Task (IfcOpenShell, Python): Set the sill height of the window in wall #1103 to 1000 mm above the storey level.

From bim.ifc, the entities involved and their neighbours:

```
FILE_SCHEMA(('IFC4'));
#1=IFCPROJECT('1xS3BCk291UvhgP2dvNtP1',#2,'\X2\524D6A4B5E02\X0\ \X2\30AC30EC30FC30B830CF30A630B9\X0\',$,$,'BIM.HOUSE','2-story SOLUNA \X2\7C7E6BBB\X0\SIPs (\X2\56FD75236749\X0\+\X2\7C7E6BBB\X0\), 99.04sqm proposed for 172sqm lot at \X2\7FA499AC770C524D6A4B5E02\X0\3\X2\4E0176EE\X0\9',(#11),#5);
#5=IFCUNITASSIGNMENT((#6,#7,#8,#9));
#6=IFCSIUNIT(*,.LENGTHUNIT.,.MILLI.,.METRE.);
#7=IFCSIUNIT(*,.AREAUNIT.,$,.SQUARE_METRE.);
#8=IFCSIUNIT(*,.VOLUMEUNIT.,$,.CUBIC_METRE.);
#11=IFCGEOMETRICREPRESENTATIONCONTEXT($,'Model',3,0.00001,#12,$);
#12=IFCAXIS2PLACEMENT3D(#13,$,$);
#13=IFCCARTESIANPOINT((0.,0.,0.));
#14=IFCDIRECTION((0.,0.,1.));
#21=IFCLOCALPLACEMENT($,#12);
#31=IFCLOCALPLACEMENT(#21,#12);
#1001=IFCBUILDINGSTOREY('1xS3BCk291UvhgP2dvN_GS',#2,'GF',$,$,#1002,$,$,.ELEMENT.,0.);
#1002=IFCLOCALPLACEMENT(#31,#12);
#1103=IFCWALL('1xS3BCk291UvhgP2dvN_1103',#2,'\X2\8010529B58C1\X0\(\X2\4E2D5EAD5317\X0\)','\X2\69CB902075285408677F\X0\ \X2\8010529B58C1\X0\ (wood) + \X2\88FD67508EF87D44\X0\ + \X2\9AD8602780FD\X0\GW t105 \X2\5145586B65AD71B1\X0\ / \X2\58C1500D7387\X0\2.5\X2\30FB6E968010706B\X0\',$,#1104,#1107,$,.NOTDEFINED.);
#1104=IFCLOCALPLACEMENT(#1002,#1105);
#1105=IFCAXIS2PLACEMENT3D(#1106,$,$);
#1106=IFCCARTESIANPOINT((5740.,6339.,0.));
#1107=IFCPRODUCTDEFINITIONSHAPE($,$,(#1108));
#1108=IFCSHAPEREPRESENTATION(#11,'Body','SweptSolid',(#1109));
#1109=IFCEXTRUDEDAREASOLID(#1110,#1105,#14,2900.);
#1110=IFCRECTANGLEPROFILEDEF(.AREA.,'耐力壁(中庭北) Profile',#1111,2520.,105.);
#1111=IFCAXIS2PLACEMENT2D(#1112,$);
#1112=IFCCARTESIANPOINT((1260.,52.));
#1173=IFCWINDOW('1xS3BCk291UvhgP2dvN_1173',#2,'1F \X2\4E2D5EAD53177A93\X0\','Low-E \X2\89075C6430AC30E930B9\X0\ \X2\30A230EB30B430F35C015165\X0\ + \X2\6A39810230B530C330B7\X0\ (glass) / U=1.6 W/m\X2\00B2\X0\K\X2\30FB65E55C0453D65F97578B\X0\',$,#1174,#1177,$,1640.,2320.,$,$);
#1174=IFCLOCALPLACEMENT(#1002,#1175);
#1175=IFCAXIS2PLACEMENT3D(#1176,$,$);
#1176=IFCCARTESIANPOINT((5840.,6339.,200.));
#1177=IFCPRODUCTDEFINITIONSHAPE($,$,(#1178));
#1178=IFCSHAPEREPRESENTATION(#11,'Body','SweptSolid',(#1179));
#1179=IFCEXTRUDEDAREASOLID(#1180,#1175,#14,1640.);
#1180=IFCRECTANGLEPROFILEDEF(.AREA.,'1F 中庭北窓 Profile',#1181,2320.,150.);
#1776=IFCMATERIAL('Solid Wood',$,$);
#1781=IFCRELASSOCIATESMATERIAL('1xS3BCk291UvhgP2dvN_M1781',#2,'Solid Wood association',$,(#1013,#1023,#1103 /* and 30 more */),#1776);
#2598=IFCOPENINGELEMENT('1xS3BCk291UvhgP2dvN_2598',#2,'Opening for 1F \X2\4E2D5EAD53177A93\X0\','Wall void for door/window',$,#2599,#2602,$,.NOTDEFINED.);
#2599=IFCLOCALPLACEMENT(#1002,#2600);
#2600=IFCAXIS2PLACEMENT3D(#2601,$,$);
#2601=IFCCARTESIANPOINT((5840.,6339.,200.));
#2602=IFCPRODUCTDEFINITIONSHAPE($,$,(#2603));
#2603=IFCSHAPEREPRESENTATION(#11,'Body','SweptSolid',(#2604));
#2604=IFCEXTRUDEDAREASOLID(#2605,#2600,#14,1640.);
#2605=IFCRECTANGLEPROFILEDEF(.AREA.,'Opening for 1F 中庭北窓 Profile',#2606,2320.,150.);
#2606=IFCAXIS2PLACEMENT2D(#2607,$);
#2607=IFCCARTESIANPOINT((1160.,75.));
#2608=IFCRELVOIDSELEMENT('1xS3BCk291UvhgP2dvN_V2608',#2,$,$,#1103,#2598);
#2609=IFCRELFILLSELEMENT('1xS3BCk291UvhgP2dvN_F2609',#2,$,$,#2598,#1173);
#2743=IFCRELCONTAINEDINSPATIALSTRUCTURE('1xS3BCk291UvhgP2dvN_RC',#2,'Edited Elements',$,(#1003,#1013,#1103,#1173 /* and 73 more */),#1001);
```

```python
import numpy as np
import ifcopenshell
import ifcopenshell.api.geometry
import ifcopenshell.geom
import ifcopenshell.util.element
import ifcopenshell.util.placement
import ifcopenshell.util.shape
import ifcopenshell.util.unit

model = ifcopenshell.open("bim.ifc")
unit_scale = ifcopenshell.util.unit.calculate_unit_scale(model)

window = model.by_guid("1xS3BCk291UvhgP2dvN_1173")
opening = window.FillsVoids[0].RelatingOpeningElement
storey = ifcopenshell.util.element.get_container(window, ifc_class="IfcBuildingStorey")
level = ifcopenshell.util.placement.get_local_placement(storey.ObjectPlacement)[2, 3]

# The opening's origin need not be at the sill, so measure its lowest point.
shape = ifcopenshell.geom.create_shape(ifcopenshell.geom.settings(), opening)
bottom = ifcopenshell.util.shape.get_shape_bottom_elevation(shape, shape.geometry) / unit_scale
dz = level + 1 / unit_scale - bottom

shift = np.array([0.0, 0.0, dz])
# The window is not placed relative to its opening, so move both.
for product in (opening, window):
    matrix = ifcopenshell.util.placement.get_local_placement(product.ObjectPlacement)
    matrix[:3, 3] += shift
    ifcopenshell.api.geometry.edit_object_placement(model, product=product, matrix=matrix, is_si=False)

print(f"moved by {dz * unit_scale:+.3f} m")

model.write("bim_rev.ifc")
```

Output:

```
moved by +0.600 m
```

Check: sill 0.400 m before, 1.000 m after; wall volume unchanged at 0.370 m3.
